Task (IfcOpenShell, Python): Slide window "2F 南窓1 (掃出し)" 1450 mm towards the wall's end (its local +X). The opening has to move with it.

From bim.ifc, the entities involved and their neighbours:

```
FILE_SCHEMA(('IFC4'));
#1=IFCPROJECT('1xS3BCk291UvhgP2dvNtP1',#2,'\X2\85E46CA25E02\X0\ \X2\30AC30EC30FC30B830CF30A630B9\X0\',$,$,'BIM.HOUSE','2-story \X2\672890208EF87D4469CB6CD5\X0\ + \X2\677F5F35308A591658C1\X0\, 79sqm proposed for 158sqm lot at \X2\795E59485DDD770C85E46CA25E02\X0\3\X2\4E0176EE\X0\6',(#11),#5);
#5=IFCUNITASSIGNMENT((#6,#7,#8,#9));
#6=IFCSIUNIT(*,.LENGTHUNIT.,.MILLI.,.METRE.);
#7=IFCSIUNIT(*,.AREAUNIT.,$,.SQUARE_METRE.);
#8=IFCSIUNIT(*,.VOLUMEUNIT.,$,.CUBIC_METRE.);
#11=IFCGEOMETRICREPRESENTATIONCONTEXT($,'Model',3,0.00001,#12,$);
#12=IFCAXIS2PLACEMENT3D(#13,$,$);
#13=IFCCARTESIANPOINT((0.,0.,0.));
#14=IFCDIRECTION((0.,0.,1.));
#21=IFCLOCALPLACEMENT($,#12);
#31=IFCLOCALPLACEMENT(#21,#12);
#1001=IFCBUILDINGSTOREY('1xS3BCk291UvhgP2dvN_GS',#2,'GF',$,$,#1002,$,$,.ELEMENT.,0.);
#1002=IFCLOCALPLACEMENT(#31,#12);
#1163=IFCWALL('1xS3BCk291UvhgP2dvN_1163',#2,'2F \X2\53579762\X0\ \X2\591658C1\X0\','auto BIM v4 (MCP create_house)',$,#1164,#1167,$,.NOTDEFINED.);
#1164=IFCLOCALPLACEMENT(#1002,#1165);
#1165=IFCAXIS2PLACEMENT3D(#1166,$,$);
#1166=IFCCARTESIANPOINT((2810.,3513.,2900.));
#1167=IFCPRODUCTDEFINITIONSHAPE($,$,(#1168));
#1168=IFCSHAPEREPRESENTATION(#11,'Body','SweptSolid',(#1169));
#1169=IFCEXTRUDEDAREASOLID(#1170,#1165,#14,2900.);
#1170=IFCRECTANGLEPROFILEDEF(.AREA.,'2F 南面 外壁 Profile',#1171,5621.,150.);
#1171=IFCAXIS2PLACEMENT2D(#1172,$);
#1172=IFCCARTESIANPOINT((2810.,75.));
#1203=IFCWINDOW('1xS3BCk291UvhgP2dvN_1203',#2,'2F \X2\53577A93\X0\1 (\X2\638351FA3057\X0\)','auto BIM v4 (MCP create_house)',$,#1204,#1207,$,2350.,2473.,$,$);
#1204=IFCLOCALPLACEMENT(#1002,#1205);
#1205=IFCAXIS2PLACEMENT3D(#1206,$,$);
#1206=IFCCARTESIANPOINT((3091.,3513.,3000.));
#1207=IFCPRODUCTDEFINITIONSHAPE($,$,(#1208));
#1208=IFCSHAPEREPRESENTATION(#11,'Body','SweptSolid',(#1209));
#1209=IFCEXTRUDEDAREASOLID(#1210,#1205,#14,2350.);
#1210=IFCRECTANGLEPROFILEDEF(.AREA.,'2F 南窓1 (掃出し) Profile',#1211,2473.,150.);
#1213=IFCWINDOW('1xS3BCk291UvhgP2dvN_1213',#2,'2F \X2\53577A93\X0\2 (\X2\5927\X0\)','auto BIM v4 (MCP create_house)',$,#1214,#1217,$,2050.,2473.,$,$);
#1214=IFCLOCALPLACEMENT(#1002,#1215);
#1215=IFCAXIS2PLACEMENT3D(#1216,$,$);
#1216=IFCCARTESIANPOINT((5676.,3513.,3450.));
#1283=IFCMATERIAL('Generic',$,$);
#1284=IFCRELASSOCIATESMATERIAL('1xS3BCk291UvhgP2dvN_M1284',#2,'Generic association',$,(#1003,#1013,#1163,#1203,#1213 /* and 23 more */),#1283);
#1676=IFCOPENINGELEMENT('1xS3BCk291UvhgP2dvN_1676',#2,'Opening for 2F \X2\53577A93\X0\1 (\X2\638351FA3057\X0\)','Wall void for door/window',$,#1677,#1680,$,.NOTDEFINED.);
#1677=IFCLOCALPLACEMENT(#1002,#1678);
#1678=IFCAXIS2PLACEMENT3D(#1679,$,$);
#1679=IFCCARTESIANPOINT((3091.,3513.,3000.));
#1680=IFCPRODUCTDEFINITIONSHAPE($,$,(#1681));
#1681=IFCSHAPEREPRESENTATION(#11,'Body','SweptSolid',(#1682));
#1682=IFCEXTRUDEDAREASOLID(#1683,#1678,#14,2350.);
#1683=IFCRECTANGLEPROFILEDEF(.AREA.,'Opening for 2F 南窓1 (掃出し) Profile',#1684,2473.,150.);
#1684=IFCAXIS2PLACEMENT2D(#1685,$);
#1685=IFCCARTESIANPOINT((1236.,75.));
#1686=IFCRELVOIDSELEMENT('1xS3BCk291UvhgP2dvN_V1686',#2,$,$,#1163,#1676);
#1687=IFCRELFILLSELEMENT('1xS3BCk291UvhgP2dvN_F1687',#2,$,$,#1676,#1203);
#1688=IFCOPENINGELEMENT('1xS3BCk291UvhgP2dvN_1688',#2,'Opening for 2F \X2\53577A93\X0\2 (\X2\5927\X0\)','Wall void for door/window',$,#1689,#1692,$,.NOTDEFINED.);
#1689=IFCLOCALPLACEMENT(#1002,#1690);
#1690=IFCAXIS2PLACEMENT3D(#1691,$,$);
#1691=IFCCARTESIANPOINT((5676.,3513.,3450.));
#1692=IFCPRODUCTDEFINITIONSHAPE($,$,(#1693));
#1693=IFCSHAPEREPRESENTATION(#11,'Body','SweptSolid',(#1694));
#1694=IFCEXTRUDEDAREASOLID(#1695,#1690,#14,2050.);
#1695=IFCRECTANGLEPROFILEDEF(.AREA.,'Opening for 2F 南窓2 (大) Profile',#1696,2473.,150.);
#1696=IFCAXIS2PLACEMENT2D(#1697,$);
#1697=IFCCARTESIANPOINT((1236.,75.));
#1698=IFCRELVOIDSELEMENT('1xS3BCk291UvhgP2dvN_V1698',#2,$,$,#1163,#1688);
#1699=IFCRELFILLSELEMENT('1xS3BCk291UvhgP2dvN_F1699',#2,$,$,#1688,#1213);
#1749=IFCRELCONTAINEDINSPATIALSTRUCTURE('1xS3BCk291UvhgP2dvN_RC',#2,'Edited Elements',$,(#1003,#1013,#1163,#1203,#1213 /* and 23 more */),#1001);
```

```python
import ifcopenshell
import ifcopenshell.api.geometry
import ifcopenshell.util.placement

model = ifcopenshell.open("bim.ifc")

window = model.by_id(1203)
opening = window.FillsVoids[0].RelatingOpeningElement
wall = opening.VoidsElements[0].RelatingBuildingElement

wall_matrix = ifcopenshell.util.placement.get_local_placement(wall.ObjectPlacement)
shift = wall_matrix[:3, 0] * 1450.0
before = ifcopenshell.util.placement.get_local_placement(window.ObjectPlacement)[:3, 3].copy()

# The window is not placed relative to its opening, so move both.
for product in (opening, window):
    matrix = ifcopenshell.util.placement.get_local_placement(product.ObjectPlacement)
    matrix[:3, 3] += shift
    ifcopenshell.api.geometry.edit_object_placement(model, product=product, matrix=matrix, is_si=False)

after = ifcopenshell.util.placement.get_local_placement(window.ObjectPlacement)[:3, 3]
print("window moved by", (after - before).round(3) + 0.0)

model.write("bim_updated.ifc")
```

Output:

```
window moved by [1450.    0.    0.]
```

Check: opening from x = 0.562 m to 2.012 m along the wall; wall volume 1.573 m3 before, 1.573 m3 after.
